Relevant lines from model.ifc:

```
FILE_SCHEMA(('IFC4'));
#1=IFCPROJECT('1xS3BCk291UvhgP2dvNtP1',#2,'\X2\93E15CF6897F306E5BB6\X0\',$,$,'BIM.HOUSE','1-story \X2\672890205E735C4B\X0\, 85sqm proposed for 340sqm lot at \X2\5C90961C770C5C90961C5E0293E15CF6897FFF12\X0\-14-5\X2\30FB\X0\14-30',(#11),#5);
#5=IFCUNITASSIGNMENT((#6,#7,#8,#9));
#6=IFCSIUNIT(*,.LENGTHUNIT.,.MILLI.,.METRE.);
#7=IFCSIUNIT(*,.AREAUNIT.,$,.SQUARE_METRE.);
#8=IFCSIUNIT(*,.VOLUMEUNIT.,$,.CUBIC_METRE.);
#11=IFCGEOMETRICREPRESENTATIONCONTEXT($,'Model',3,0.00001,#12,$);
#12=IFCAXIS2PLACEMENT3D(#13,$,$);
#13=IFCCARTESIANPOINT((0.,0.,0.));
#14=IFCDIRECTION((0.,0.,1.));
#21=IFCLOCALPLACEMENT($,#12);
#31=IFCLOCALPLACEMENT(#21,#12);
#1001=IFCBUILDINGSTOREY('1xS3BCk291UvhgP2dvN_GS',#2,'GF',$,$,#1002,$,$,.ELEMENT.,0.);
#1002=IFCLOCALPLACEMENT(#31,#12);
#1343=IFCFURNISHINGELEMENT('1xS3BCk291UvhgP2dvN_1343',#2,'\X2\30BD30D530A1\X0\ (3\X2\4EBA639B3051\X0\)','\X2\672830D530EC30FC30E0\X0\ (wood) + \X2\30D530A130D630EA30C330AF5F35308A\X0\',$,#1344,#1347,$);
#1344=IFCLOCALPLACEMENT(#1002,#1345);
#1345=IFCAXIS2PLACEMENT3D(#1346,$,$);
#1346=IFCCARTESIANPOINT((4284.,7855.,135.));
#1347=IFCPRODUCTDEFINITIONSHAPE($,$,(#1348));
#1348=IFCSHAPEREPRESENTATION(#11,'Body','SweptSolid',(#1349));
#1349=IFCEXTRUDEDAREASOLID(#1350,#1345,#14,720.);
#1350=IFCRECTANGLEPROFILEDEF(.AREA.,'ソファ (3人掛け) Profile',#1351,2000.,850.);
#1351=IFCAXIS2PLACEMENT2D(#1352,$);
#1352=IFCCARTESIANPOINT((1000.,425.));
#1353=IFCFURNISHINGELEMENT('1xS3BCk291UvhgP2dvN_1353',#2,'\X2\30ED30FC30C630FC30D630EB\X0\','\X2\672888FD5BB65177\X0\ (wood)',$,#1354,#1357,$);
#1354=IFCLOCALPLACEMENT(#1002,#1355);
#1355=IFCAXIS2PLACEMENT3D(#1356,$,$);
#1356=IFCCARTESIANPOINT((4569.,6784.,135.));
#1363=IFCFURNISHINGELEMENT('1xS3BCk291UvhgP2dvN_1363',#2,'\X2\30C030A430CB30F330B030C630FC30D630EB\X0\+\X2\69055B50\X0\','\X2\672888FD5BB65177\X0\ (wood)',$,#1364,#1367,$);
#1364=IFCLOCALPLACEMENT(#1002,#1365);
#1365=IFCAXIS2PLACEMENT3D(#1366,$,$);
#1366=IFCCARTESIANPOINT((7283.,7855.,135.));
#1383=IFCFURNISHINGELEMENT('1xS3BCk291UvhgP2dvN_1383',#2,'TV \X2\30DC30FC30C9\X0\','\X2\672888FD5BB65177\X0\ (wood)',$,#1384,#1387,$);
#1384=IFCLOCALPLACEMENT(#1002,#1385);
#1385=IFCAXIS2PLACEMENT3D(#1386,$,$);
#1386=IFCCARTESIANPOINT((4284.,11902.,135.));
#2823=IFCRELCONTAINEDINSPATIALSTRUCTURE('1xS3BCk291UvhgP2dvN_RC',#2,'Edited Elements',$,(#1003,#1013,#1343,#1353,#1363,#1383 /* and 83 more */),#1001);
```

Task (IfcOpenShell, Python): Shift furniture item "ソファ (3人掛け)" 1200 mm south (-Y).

```python
import ifcopenshell
import ifcopenshell.api.geometry
import ifcopenshell.util.placement
import ifcopenshell.util.unit

model = ifcopenshell.open("model.ifc")
unit_scale = ifcopenshell.util.unit.calculate_unit_scale(model)

item = model.by_id(1343)
matrix = ifcopenshell.util.placement.get_local_placement(item.ObjectPlacement)
matrix[1, 3] -= 1.2 / unit_scale
ifcopenshell.api.geometry.edit_object_placement(model, product=item, matrix=matrix, is_si=False)

print(ifcopenshell.util.placement.get_local_placement(item.ObjectPlacement).round(3) + 0.0)

model.write("model_updated.ifc")
```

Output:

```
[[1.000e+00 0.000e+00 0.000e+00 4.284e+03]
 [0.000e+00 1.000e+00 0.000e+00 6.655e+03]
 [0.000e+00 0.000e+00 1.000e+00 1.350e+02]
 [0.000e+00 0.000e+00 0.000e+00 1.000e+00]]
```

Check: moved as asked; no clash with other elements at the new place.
